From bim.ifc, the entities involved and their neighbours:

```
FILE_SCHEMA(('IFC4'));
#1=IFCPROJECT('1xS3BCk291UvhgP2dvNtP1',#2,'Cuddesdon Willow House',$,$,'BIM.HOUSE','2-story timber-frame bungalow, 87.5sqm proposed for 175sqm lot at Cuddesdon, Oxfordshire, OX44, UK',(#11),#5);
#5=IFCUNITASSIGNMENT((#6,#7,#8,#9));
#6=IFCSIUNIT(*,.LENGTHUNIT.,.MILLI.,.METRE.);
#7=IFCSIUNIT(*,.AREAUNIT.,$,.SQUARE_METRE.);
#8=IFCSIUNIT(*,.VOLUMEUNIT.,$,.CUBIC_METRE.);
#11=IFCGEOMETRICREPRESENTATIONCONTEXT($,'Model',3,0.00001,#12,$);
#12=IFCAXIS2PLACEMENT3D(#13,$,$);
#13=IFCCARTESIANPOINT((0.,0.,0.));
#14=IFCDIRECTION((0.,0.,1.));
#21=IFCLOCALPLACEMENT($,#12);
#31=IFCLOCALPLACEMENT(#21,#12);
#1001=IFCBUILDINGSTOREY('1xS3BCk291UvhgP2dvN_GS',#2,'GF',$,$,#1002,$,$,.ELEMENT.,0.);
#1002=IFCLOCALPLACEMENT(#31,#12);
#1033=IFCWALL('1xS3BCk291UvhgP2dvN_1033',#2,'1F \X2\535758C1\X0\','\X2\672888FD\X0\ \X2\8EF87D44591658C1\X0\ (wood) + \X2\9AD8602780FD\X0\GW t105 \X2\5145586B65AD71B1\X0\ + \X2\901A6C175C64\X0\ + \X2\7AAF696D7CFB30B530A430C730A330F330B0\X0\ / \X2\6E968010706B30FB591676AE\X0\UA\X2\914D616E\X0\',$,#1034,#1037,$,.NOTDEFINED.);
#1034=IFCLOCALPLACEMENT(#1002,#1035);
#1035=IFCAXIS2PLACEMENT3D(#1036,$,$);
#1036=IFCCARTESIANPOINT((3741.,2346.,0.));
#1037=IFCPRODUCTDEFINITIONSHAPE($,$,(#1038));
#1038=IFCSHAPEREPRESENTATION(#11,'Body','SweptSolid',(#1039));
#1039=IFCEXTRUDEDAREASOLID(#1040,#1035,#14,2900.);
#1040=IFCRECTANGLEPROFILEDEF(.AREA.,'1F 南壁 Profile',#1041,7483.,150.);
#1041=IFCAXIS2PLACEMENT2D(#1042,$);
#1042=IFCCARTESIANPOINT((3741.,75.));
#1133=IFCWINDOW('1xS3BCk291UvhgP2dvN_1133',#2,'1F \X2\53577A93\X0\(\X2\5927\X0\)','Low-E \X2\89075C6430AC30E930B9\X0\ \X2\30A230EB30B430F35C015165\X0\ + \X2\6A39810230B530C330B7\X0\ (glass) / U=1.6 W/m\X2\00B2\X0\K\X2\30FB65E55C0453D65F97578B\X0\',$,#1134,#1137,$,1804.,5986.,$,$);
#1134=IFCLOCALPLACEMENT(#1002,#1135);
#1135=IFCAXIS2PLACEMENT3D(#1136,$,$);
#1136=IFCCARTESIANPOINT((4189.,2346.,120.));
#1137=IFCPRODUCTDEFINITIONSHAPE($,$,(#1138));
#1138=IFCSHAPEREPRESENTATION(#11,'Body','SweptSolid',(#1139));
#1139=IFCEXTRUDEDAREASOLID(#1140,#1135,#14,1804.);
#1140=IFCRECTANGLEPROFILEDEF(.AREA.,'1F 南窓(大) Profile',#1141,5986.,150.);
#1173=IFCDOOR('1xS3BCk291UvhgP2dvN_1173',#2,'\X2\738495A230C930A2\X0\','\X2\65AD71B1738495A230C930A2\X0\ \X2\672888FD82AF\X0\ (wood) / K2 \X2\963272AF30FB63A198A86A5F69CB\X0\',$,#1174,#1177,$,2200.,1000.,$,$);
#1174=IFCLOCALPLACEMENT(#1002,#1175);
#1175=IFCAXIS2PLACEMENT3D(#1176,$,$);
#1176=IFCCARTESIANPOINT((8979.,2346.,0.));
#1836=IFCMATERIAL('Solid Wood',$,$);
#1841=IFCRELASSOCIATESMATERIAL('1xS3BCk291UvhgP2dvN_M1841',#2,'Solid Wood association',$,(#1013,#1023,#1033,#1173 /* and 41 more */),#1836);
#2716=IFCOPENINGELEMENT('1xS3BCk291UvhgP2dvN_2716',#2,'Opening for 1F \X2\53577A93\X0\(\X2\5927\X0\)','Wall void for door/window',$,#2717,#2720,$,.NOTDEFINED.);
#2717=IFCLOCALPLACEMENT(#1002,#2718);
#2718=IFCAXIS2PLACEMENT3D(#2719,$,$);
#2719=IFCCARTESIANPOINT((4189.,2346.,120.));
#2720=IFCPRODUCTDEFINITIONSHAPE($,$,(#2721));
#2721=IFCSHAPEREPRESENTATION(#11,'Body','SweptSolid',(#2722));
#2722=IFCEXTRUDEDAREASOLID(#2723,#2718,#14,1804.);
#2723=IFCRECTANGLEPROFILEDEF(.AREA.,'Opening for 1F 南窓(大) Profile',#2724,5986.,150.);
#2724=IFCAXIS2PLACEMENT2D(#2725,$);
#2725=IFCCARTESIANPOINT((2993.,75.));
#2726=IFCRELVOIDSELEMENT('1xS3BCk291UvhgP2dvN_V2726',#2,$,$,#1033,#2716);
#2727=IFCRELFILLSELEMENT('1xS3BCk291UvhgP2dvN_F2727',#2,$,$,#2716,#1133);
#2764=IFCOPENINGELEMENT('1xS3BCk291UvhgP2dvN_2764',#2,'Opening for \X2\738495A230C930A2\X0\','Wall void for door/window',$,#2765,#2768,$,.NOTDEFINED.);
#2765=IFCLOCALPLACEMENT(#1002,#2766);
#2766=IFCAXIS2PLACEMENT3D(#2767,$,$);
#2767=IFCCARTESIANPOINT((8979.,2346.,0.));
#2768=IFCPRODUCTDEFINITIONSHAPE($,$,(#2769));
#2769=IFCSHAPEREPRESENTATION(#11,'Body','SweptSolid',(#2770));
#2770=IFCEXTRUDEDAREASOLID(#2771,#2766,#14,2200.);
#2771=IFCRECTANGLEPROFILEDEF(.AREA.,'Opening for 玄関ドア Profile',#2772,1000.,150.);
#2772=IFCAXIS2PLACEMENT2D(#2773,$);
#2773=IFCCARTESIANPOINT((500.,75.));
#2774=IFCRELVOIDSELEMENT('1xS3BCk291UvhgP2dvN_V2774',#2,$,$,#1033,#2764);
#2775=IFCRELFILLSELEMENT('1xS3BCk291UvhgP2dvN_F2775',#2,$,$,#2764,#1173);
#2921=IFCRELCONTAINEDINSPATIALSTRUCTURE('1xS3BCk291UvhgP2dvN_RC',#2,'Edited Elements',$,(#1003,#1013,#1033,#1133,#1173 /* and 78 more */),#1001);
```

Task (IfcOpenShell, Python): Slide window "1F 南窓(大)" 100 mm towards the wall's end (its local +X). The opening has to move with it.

```python
import ifcopenshell
import ifcopenshell.api.geometry
import ifcopenshell.util.placement
import ifcopenshell.util.unit

model = ifcopenshell.open("bim.ifc")
unit_scale = ifcopenshell.util.unit.calculate_unit_scale(model)

window = model.by_id(1133)
opening = window.FillsVoids[0].RelatingOpeningElement
wall = opening.VoidsElements[0].RelatingBuildingElement

wall_matrix = ifcopenshell.util.placement.get_local_placement(wall.ObjectPlacement)
shift = wall_matrix[:3, 0] * 0.1 / unit_scale
before = ifcopenshell.util.placement.get_local_placement(window.ObjectPlacement)[:3, 3].copy()

# The window is not placed relative to its opening, so move both.
for product in (opening, window):
    matrix = ifcopenshell.util.placement.get_local_placement(product.ObjectPlacement)
    matrix[:3, 3] += shift
    ifcopenshell.api.geometry.edit_object_placement(model, product=product, matrix=matrix, is_si=False)

after = ifcopenshell.util.placement.get_local_placement(window.ObjectPlacement)[:3, 3]
print("window moved by", (after - before).round(3) + 0.0)

model.write("bim_edited.ifc")
```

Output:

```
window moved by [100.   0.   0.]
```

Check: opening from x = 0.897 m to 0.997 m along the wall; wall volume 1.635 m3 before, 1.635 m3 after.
